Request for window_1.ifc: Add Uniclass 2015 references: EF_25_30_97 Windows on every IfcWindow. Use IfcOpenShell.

First a look at what the model holds.

```python
import ifcopenshell

model = ifcopenshell.open("window_1.ifc")
print(model.schema)
print("classifications:", [c.Name for c in model.by_type("IfcClassification")])
for ifc_class in ("IfcDoor", "IfcRoof", "IfcStair", "IfcWall", "IfcWindow"):
    print(ifc_class, len(model.by_type(ifc_class)))
```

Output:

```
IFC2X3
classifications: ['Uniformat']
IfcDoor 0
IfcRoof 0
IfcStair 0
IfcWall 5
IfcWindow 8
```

```python
import ifcopenshell
import ifcopenshell.api.classification

model = ifcopenshell.open("window_1.ifc")

# IFC2X3 requires Source and Edition and has no link from the project to the system.
system = model.create_entity("IfcClassification", Source="NBS", Edition="2015", Name="Uniclass 2015")

codes = {
    "IfcWindow": ("EF_25_30_97", "Windows"),
}
for ifc_class, (code, name) in codes.items():
    products = model.by_type(ifc_class)
    ifcopenshell.api.classification.add_reference(
        model, products=products, classification=system, identification=code, name=name
    )
    print(code, len(products))

model.write("window_1_edited.ifc")
```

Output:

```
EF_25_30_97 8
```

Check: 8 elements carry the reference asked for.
